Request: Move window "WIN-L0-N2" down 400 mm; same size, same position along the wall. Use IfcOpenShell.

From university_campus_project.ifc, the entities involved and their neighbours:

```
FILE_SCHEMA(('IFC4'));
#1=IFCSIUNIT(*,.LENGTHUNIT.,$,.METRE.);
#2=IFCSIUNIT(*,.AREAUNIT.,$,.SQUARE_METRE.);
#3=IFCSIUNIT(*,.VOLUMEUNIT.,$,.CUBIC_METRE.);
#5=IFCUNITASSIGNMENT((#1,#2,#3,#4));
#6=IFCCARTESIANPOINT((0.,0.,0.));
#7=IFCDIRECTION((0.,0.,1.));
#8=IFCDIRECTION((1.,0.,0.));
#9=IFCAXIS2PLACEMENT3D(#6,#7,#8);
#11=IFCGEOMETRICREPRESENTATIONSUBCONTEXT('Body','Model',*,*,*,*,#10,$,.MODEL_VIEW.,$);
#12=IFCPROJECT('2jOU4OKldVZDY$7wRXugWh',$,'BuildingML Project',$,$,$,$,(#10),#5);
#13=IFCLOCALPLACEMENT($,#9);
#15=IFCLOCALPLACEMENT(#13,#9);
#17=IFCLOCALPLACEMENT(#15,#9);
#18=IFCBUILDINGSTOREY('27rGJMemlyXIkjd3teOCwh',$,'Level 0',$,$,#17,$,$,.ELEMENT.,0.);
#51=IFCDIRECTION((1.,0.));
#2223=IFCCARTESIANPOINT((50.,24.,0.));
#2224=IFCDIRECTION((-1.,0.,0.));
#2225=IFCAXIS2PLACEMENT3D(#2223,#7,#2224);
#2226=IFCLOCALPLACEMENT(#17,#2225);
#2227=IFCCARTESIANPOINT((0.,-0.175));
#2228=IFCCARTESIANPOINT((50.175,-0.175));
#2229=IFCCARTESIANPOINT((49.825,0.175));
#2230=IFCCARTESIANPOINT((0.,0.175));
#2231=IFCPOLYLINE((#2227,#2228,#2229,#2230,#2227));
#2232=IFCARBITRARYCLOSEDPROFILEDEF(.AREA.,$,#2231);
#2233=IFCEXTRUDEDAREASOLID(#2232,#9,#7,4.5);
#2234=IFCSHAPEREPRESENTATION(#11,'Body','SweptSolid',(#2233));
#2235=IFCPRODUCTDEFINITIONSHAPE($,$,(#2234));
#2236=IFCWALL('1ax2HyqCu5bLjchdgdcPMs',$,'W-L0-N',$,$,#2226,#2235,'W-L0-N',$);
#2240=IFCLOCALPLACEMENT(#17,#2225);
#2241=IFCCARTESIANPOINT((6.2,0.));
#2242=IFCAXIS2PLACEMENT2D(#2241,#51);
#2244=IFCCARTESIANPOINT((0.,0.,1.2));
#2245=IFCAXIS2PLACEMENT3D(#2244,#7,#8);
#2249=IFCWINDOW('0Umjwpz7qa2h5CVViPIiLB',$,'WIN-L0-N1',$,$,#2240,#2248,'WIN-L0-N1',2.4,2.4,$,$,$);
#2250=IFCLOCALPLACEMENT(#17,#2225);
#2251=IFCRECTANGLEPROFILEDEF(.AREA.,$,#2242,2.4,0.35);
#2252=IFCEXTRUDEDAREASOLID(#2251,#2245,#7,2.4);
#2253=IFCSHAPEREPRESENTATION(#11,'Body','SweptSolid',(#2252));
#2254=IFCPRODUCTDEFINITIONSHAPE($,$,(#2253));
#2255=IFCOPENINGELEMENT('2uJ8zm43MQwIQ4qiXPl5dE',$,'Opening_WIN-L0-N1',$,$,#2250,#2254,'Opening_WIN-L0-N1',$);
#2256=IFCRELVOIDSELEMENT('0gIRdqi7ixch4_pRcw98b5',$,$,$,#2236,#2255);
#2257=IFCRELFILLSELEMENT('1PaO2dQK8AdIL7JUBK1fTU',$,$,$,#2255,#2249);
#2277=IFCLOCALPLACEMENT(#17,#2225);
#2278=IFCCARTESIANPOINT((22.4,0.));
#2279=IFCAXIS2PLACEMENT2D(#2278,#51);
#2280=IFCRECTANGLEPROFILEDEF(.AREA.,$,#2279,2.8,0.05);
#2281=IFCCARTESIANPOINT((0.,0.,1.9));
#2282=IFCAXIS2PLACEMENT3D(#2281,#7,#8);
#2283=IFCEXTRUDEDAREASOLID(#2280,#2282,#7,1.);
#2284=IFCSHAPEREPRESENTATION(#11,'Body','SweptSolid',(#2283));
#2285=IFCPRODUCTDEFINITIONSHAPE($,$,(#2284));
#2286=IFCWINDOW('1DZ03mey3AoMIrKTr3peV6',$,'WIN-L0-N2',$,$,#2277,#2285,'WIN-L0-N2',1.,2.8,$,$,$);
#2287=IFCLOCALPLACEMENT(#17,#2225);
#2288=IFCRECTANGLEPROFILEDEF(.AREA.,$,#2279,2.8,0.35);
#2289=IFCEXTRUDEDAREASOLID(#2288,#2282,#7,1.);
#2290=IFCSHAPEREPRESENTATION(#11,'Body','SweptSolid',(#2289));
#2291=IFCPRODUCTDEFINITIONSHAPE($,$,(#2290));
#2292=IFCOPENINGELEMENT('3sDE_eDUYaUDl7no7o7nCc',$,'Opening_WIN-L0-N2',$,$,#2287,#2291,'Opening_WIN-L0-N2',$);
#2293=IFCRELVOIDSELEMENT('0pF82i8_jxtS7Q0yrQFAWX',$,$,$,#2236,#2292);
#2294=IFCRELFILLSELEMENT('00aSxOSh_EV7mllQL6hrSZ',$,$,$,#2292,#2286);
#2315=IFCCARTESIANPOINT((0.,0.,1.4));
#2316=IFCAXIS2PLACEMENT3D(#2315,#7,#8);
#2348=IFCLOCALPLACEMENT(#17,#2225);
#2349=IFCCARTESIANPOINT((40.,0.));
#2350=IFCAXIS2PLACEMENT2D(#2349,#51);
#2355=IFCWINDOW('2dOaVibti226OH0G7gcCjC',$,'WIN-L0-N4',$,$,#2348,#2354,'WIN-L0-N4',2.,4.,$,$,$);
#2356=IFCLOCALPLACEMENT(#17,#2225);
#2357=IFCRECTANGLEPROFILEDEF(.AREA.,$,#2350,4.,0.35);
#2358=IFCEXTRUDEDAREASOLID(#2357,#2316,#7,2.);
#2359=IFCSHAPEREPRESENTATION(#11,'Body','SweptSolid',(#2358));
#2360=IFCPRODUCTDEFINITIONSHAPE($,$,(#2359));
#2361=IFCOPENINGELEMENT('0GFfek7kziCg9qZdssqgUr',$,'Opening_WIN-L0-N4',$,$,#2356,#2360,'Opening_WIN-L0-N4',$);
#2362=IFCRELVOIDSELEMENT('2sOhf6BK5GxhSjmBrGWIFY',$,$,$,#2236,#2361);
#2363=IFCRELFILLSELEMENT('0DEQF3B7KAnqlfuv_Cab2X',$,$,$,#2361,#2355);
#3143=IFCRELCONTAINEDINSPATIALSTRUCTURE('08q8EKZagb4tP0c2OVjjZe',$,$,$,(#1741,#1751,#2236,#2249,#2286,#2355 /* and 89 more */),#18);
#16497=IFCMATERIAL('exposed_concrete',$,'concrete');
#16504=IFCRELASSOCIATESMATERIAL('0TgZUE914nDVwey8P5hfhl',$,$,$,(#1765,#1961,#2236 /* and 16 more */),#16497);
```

```python
import numpy as np
import ifcopenshell
import ifcopenshell.api.geometry
import ifcopenshell.util.placement
import ifcopenshell.util.unit

model = ifcopenshell.open("university_campus_project.ifc")
unit_scale = ifcopenshell.util.unit.calculate_unit_scale(model)

window = model.by_guid("1DZ03mey3AoMIrKTr3peV6")
opening = window.FillsVoids[0].RelatingOpeningElement
dz = -0.4 / unit_scale

shift = np.array([0.0, 0.0, dz])
# The window is not placed relative to its opening, so move both.
for product in (opening, window):
    matrix = ifcopenshell.util.placement.get_local_placement(product.ObjectPlacement)
    matrix[:3, 3] += shift
    ifcopenshell.api.geometry.edit_object_placement(model, product=product, matrix=matrix, is_si=False)

print(f"moved by {dz * unit_scale:+.3f} m")

model.write("university_campus_project-out.ifc")
```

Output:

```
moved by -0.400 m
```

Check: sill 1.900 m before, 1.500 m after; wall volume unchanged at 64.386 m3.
